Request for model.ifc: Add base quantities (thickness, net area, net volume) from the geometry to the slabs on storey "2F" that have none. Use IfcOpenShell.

First a look at what the model holds.

```python
import ifcopenshell
import ifcopenshell.util.element
import ifcopenshell.util.unit

model = ifcopenshell.open("model.ifc")
print(model.schema)
for unit_type in ("LENGTHUNIT", "AREAUNIT", "VOLUMEUNIT"):
    print(unit_type, ifcopenshell.util.unit.calculate_unit_scale(model, unit_type))
storey = next(s for s in model.by_type("IfcBuildingStorey") if s.Name == "2F")
slabs = [e for e in ifcopenshell.util.element.get_decomposition(storey) if e.is_a("IfcSlab")]
for e in sorted(slabs, key=lambda e: e.id()):
    print(e.id(), e.is_a(), e.Name, list(ifcopenshell.util.element.get_psets(e, qtos_only=True)), sep=" | ")
```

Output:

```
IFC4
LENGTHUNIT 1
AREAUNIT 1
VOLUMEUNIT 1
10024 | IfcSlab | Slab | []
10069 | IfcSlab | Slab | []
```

```python
import ifcopenshell
import ifcopenshell.api.pset
import ifcopenshell.geom
import ifcopenshell.util.element
import ifcopenshell.util.shape
import ifcopenshell.util.unit

model = ifcopenshell.open("model.ifc")
unit_scale = ifcopenshell.util.unit.calculate_unit_scale(model)
area_scale = ifcopenshell.util.unit.calculate_unit_scale(model, "AREAUNIT")
volume_scale = ifcopenshell.util.unit.calculate_unit_scale(model, "VOLUMEUNIT")
settings = ifcopenshell.geom.settings()

storey = next(s for s in model.by_type("IfcBuildingStorey") if s.Name == "2F")
slabs = [e for e in ifcopenshell.util.element.get_decomposition(storey) if e.is_a("IfcSlab")]

for e in sorted(slabs, key=lambda e: e.id()):
    if ifcopenshell.util.element.get_psets(e, qtos_only=True, should_inherit=False):
        continue
    # Geometry comes back in metres, in the element's own axes.
    shape = ifcopenshell.geom.create_shape(settings, e)
    values = {
        "Width": ifcopenshell.util.shape.get_z(shape.geometry) / unit_scale,
        "NetArea": ifcopenshell.util.shape.get_footprint_area(shape.geometry) / area_scale,
        "NetVolume": ifcopenshell.util.shape.get_volume(shape.geometry) / volume_scale,
    }
    qto = ifcopenshell.api.pset.add_qto(model, product=e, name="Qto_SlabBaseQuantities")
    ifcopenshell.api.pset.edit_qto(model, qto=qto, properties=values)
    print(e.id(), {k: round(v, 3) for k, v in values.items()})

model.write("model_updated.ifc")
```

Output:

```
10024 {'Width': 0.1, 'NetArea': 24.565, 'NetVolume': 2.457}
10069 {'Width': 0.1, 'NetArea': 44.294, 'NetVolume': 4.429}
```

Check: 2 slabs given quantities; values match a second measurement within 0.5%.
